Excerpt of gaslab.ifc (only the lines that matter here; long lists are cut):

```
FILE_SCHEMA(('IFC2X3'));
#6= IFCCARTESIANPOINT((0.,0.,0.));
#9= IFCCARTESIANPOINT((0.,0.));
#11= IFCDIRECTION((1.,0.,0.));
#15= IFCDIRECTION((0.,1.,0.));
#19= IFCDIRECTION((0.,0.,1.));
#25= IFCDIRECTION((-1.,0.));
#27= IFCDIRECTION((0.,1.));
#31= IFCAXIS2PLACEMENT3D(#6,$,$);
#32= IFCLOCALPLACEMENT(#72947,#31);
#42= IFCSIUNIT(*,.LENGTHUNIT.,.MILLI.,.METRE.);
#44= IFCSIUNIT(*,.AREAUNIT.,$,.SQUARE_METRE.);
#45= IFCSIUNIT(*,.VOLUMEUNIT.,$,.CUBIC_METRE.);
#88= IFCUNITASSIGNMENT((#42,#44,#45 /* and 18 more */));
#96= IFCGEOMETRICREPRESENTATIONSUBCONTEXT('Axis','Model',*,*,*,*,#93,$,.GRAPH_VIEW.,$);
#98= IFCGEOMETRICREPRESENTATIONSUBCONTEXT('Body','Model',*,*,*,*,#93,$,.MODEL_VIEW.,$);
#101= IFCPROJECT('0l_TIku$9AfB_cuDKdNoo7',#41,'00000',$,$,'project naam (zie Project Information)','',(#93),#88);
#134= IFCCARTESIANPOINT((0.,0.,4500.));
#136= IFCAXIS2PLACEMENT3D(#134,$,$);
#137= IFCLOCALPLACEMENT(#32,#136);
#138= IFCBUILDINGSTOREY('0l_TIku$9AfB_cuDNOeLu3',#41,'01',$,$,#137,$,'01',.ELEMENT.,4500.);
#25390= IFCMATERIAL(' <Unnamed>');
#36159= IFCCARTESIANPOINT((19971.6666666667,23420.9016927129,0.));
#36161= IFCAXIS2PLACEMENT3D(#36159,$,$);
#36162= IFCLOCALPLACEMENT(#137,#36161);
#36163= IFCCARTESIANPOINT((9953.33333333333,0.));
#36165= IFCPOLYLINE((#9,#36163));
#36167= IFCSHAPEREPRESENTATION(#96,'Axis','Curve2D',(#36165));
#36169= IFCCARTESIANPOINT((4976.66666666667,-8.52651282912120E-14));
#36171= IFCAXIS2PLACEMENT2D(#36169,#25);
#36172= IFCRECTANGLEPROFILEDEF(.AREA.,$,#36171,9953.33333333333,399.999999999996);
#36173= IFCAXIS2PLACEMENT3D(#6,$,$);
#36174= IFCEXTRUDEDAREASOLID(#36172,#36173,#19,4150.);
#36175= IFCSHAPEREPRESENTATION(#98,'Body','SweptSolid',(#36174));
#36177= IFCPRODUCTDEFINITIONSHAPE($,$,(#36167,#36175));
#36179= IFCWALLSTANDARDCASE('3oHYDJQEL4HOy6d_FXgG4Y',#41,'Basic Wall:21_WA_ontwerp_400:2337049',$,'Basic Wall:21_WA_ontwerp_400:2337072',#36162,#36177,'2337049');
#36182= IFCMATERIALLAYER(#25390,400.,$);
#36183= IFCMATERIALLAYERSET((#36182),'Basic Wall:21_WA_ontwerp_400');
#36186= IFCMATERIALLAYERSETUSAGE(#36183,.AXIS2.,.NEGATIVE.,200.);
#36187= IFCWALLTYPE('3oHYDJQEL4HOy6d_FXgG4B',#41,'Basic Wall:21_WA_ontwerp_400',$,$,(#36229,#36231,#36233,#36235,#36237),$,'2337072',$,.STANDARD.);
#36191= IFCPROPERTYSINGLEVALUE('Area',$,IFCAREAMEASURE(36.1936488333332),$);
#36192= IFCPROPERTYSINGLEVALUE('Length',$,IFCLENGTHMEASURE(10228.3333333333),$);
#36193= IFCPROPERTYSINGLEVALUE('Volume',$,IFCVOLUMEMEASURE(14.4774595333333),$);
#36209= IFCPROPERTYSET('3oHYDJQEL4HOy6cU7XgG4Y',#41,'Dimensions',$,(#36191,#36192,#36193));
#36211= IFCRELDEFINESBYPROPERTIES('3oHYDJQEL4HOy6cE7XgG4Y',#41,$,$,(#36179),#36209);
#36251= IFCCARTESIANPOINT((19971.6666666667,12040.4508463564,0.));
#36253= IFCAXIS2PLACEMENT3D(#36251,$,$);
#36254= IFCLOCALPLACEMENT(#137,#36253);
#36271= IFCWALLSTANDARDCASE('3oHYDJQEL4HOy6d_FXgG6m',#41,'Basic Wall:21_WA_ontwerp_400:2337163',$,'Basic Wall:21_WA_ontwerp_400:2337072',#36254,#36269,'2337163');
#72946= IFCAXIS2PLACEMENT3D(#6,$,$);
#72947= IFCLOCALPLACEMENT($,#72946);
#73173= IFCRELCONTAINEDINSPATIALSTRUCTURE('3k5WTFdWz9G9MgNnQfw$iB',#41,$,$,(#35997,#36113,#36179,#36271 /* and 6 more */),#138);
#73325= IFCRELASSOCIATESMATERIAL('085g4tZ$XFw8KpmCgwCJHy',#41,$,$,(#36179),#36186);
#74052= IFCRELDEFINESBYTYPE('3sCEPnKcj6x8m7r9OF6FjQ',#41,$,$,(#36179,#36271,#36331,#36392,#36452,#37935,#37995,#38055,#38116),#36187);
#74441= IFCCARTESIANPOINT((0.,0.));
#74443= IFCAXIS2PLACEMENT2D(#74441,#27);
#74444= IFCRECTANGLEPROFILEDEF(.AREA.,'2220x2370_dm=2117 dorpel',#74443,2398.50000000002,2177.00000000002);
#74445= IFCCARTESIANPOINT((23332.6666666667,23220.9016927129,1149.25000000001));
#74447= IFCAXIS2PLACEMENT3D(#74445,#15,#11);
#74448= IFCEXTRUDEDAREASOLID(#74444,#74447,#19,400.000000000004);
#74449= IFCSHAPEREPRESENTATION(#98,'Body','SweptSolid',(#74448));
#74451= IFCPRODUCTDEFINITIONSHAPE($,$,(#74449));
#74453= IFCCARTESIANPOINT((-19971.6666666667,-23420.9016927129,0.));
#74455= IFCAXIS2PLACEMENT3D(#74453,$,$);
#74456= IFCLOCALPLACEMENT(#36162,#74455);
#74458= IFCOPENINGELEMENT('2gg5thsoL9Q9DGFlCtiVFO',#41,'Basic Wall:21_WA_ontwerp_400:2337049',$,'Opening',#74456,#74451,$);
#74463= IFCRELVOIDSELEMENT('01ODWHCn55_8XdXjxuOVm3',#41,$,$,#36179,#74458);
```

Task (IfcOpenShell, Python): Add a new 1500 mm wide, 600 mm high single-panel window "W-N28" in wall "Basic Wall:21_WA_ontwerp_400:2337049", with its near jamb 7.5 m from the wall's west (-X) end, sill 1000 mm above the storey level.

```python
import numpy as np
import ifcopenshell
import ifcopenshell.api.feature
import ifcopenshell.api.geometry
import ifcopenshell.api.pset
import ifcopenshell.api.root
import ifcopenshell.api.spatial
import ifcopenshell.api.type
import ifcopenshell.geom
import ifcopenshell.util.element
import ifcopenshell.util.placement
import ifcopenshell.util.representation
import ifcopenshell.util.shape
import ifcopenshell.util.unit

model = ifcopenshell.open("gaslab.ifc")
unit_scale = ifcopenshell.util.unit.calculate_unit_scale(model)
area_scale = ifcopenshell.util.unit.calculate_unit_scale(model, "AREAUNIT")
volume_scale = ifcopenshell.util.unit.calculate_unit_scale(model, "VOLUMEUNIT")
settings = ifcopenshell.geom.settings()


def volume(element):
    """Net volume in cubic metres, openings subtracted."""
    shape = ifcopenshell.geom.create_shape(settings, element)
    return ifcopenshell.util.shape.get_volume(shape.geometry)


wall = model.by_id(36179)
storey = ifcopenshell.util.element.get_container(wall, ifc_class="IfcBuildingStorey")
context = ifcopenshell.util.representation.get_context(model, "Model", "Body", "MODEL_VIEW")
before = volume(wall)

width, height, from_end, sill = 1.5, 0.6, 7.5, 1  # metres

# The wall runs along its own X axis, and the end named is its -X end.
wall_shape = ifcopenshell.geom.create_shape(settings, wall)
x, y, z = ifcopenshell.util.shape.get_vertices(wall_shape.geometry).T
start = x.min() + from_end
face, thickness = float(y.min()), float(y.max() - y.min())
wall_matrix = ifcopenshell.util.placement.get_local_placement(wall.ObjectPlacement)
level = ifcopenshell.util.placement.get_local_placement(storey.ObjectPlacement)[2, 3]


def in_wall(x, y):
    """Placement at x, y metres in the wall's axes, at sill height."""
    matrix = wall_matrix.copy()
    matrix[:, 3] = wall_matrix @ np.array([x / unit_scale, y / unit_scale, 0.0, 1.0])
    matrix[2, 3] = level + sill / unit_scale
    return matrix


# Opening: a box that overshoots both wall faces by 50 mm.
opening = ifcopenshell.api.root.create_entity(model, ifc_class="IfcOpeningElement")
box = ifcopenshell.api.geometry.add_wall_representation(
    model, context=context, length=width, height=height, thickness=thickness + 0.1
)
ifcopenshell.api.geometry.assign_representation(model, product=opening, representation=box)
ifcopenshell.api.geometry.edit_object_placement(model, product=opening, matrix=in_wall(start, face - 0.05), is_si=False)
ifcopenshell.api.feature.add_feature(model, feature=opening, element=wall)

window = ifcopenshell.api.root.create_entity(model, ifc_class="IfcWindow", name="W-N28")
window.OverallWidth, window.OverallHeight = width / unit_scale, height / unit_scale
body = ifcopenshell.api.geometry.add_window_representation(
    model,
    context=context,
    overall_width=window.OverallWidth,
    overall_height=window.OverallHeight,
    partition_type="SINGLE_PANEL",
)
ifcopenshell.api.geometry.assign_representation(model, product=window, representation=body)
ifcopenshell.api.spatial.assign_container(model, products=[window], relating_structure=storey)
fills = ifcopenshell.api.feature.add_filling(model, opening=opening, element=window)
fills.OwnerHistory = window.OwnerHistory  # required in IFC2X3

# IFC2X3 keeps the operation on the window style.
style = ifcopenshell.api.root.create_entity(model, ifc_class="IfcWindowStyle", name="W-N28")
style.OperationType, style.ConstructionType = "SINGLE_PANEL", "NOTDEFINED"
style.ParameterTakesPrecedence = style.Sizeable = False
ifcopenshell.api.type.assign_type(model, related_objects=[window], relating_type=style)

# Centre the window in the wall's thickness.
ifcopenshell.api.geometry.edit_object_placement(model, product=window, matrix=in_wall(start, face), is_si=False)
window_shape = ifcopenshell.geom.create_shape(settings, window)
depth = ifcopenshell.util.shape.get_vertices(window_shape.geometry)[:, 1]
offset = face + thickness / 2 - (depth.min() + depth.max()) / 2
ifcopenshell.api.geometry.edit_object_placement(model, product=window, matrix=in_wall(start, offset), is_si=False)

after = volume(wall)

# Update the wall's stored quantities.
pset = model.by_id(ifcopenshell.util.element.get_pset(wall, "Dimensions", should_inherit=False)["id"])
ifcopenshell.api.pset.edit_pset(model, pset=pset, properties={
    "Area": model.create_entity("IfcAreaMeasure", after / thickness / area_scale),
    "Volume": model.create_entity("IfcVolumeMeasure", after / volume_scale),
})

print(f"wall volume {before:.3f} -> {after:.3f} m3")

model.write("gaslab_edited.ifc")
```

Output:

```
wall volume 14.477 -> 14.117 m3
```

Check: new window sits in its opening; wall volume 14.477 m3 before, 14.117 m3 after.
